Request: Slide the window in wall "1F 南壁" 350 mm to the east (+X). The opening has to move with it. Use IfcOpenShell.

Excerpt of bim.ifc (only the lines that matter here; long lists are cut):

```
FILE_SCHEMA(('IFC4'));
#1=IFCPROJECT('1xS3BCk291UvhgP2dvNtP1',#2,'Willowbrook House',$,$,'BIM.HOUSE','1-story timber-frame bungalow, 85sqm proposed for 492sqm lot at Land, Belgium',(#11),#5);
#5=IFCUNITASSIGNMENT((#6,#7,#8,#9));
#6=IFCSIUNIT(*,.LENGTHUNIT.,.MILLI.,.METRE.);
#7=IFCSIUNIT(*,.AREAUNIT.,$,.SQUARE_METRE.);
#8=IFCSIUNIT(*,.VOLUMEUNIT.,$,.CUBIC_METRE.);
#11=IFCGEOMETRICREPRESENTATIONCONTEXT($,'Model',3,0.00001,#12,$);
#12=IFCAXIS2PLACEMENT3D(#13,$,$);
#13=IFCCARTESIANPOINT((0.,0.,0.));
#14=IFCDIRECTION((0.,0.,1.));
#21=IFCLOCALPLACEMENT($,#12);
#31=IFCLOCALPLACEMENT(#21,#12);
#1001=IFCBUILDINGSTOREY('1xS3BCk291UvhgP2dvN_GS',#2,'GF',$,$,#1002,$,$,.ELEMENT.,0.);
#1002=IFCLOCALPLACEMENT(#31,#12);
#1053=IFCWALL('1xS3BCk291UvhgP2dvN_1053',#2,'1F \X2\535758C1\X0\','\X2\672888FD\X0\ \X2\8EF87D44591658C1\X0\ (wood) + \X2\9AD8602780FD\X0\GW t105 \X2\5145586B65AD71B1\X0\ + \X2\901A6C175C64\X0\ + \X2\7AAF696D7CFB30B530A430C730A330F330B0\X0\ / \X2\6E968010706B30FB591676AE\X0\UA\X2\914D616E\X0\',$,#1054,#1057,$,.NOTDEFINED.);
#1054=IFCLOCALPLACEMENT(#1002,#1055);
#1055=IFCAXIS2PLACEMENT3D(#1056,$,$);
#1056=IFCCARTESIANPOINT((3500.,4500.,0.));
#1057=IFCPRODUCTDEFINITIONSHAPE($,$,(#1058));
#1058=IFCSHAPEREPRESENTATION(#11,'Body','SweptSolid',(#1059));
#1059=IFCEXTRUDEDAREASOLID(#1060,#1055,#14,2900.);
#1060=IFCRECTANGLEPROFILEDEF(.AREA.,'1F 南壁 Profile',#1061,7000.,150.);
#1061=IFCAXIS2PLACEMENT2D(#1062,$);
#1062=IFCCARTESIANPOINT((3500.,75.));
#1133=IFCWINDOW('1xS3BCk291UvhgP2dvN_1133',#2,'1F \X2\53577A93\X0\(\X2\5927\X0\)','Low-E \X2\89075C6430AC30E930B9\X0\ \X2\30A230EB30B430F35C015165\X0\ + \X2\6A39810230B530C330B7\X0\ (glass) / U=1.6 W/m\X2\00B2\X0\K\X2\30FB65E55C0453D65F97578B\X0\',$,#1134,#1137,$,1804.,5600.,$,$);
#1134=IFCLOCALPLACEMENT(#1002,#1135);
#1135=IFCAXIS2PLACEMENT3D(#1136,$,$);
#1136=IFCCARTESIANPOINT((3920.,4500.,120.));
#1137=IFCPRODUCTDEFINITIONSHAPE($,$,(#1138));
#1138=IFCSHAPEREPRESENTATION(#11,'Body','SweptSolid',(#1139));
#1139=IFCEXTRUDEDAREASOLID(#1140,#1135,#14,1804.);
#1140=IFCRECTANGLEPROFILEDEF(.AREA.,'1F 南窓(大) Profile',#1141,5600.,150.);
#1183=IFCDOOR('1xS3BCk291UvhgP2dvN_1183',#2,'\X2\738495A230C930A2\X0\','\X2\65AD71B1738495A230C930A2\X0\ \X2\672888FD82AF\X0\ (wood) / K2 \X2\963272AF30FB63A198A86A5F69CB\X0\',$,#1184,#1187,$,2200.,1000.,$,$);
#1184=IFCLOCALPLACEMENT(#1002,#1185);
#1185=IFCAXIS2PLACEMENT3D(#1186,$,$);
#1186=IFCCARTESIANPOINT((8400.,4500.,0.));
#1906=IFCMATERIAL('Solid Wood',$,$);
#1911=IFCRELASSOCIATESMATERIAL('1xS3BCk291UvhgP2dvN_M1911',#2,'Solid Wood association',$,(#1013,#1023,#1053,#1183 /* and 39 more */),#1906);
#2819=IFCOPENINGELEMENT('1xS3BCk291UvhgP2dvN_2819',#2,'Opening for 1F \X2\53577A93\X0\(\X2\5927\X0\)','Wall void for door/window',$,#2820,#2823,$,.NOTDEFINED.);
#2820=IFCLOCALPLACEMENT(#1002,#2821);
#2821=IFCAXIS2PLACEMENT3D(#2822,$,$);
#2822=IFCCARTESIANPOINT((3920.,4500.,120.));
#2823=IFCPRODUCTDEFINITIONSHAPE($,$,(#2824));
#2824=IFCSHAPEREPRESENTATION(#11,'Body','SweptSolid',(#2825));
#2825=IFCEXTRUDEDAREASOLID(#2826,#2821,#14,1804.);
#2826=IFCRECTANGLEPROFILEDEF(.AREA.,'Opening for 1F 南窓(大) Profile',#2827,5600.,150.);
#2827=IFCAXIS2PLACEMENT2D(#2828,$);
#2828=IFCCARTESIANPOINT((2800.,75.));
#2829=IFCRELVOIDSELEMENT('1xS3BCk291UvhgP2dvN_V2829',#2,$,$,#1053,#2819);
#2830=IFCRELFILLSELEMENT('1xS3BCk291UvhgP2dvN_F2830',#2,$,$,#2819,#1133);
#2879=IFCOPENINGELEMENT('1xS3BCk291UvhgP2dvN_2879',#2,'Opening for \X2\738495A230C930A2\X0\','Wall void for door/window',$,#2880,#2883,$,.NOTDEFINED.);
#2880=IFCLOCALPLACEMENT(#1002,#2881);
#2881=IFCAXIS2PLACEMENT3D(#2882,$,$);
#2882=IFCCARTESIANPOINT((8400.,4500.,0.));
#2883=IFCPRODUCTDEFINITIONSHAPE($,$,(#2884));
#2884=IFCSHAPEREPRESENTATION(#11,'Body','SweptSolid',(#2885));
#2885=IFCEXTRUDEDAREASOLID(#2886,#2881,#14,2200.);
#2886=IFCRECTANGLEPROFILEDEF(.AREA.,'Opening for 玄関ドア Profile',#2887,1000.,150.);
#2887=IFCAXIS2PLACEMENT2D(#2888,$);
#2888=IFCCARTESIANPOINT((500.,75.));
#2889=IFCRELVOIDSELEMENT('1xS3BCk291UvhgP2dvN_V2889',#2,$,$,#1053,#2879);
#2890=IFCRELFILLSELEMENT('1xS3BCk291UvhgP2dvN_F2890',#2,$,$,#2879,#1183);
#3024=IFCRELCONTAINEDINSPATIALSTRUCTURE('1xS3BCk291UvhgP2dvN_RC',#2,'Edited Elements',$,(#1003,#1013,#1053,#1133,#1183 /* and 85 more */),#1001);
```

```python
import ifcopenshell
import ifcopenshell.api.geometry
import ifcopenshell.util.placement

model = ifcopenshell.open("bim.ifc")

window = model.by_id(1133)
opening = window.FillsVoids[0].RelatingOpeningElement
wall = opening.VoidsElements[0].RelatingBuildingElement

wall_matrix = ifcopenshell.util.placement.get_local_placement(wall.ObjectPlacement)
shift = wall_matrix[:3, 0] * 350.0
before = ifcopenshell.util.placement.get_local_placement(window.ObjectPlacement)[:3, 3].copy()

# The window is not placed relative to its opening, so move both.
for product in (opening, window):
    matrix = ifcopenshell.util.placement.get_local_placement(product.ObjectPlacement)
    matrix[:3, 3] += shift
    ifcopenshell.api.geometry.edit_object_placement(model, product=product, matrix=matrix, is_si=False)

after = ifcopenshell.util.placement.get_local_placement(window.ObjectPlacement)[:3, 3]
print("window moved by", (after - before).round(3) + 0.0)

model.write("bim-out.ifc")
```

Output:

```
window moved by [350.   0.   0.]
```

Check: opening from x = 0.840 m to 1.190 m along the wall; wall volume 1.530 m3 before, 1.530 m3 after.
